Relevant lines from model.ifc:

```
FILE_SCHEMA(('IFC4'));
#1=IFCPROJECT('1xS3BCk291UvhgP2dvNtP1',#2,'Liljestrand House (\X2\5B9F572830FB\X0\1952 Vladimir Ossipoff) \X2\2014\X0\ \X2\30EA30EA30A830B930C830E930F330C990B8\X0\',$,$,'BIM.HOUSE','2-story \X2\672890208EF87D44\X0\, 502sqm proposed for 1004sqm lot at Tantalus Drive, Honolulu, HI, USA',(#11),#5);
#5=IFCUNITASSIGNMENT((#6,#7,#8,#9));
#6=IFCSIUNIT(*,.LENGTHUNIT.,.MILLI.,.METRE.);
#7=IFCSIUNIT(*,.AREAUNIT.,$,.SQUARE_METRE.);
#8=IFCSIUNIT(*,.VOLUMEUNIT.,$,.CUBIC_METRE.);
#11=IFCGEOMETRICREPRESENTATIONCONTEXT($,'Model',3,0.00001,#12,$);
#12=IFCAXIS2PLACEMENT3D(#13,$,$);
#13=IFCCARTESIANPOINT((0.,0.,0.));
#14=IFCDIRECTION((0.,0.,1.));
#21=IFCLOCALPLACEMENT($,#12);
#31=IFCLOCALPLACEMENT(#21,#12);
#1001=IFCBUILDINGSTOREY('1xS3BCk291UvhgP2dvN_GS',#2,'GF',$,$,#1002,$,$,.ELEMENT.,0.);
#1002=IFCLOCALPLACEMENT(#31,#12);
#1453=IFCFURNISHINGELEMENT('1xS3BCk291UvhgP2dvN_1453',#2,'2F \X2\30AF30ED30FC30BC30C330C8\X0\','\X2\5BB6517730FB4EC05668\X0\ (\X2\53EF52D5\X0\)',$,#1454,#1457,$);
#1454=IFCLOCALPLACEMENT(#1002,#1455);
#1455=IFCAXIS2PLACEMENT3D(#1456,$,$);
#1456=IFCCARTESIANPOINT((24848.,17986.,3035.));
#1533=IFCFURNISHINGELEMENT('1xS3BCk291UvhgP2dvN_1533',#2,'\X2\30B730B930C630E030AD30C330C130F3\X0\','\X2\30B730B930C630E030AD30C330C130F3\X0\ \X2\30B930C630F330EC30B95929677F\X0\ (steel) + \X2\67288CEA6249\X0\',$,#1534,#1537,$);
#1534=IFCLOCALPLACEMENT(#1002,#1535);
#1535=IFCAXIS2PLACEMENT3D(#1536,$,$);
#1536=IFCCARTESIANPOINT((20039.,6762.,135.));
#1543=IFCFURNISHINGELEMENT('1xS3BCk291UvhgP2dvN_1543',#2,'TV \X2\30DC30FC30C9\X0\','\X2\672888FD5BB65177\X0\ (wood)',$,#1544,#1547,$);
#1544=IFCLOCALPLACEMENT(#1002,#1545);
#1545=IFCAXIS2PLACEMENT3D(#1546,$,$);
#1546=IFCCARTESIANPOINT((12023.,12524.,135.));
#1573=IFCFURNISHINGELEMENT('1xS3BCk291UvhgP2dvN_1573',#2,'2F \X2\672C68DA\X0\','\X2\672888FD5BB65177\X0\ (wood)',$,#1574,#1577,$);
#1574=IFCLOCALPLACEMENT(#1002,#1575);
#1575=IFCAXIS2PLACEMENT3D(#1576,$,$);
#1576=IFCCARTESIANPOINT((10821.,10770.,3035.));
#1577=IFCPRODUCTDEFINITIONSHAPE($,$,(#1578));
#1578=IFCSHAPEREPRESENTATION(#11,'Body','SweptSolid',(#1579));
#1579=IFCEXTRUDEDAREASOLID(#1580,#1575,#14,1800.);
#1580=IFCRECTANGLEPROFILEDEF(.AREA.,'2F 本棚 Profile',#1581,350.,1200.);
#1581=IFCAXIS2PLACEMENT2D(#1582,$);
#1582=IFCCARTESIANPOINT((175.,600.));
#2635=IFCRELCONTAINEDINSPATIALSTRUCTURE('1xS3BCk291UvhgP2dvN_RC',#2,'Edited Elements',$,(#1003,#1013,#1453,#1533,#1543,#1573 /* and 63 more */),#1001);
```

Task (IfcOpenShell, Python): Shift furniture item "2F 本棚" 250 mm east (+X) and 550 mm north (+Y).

```python
import ifcopenshell
import ifcopenshell.api.geometry
import ifcopenshell.util.placement

model = ifcopenshell.open("model.ifc")

item = model.by_guid("1xS3BCk291UvhgP2dvN_1573")
matrix = ifcopenshell.util.placement.get_local_placement(item.ObjectPlacement)
matrix[0, 3] += 250.0
matrix[1, 3] += 550.0
ifcopenshell.api.geometry.edit_object_placement(model, product=item, matrix=matrix, is_si=False)

print(ifcopenshell.util.placement.get_local_placement(item.ObjectPlacement).round(3) + 0.0)

model.write("model_v2.ifc")
```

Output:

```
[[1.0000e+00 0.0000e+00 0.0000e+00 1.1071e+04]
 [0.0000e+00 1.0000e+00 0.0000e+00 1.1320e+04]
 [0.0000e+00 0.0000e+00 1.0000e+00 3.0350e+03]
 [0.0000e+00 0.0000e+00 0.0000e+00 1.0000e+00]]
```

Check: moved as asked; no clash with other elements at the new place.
